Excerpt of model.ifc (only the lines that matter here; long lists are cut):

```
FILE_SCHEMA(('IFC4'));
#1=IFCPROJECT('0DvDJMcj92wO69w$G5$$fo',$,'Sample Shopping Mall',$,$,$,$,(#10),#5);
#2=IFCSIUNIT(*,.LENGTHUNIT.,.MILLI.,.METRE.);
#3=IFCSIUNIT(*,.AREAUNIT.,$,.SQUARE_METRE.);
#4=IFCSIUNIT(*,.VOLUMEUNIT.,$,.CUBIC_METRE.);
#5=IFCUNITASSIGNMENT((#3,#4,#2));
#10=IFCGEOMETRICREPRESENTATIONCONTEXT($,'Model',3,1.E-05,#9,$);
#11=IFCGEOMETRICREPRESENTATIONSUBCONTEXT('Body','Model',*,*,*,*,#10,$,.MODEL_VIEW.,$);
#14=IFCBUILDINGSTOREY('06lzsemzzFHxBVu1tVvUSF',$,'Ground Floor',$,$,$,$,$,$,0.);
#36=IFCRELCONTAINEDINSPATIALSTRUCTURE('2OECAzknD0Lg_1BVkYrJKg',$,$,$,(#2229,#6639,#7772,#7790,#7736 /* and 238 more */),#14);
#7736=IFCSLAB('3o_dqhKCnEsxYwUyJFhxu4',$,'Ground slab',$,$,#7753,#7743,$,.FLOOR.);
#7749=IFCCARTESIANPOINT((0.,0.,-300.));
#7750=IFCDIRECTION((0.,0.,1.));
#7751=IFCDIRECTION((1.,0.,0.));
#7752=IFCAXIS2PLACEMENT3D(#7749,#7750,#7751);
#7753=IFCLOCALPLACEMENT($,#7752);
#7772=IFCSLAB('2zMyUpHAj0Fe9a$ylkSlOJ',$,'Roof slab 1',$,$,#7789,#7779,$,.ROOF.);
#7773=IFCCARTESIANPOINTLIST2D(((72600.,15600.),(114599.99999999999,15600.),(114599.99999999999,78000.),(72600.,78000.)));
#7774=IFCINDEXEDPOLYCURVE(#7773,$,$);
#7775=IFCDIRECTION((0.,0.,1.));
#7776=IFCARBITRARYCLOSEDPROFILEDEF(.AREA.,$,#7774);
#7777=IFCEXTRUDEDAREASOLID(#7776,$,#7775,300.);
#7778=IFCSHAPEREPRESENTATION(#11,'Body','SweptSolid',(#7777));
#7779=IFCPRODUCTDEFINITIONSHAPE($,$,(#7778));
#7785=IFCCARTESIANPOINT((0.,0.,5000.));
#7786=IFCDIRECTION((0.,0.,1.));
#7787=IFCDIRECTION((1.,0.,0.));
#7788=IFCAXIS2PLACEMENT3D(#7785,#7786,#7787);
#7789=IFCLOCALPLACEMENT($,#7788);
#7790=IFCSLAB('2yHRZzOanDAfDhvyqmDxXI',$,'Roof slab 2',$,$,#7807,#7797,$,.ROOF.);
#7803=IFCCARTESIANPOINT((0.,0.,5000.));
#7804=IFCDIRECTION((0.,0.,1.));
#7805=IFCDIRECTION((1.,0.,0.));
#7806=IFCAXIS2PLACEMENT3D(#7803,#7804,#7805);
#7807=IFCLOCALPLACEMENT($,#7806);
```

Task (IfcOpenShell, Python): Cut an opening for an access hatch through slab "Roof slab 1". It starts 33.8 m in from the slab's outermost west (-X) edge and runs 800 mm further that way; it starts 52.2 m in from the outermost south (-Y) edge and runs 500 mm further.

```python
import numpy as np
import ifcopenshell
import ifcopenshell.api.feature
import ifcopenshell.api.geometry
import ifcopenshell.api.root
import ifcopenshell.geom
import ifcopenshell.util.placement
import ifcopenshell.util.representation
import ifcopenshell.util.shape
import ifcopenshell.util.unit

model = ifcopenshell.open("model.ifc")
unit_scale = ifcopenshell.util.unit.calculate_unit_scale(model)
settings = ifcopenshell.geom.settings()


def volume(element):
    """Net volume in cubic metres, openings subtracted."""
    shape = ifcopenshell.geom.create_shape(settings, element)
    return ifcopenshell.util.shape.get_volume(shape.geometry)


slab = model.by_guid("2zMyUpHAj0Fe9a$ylkSlOJ")
before = volume(slab)

# Extent in the slab's own axes, in metres. The edges named are its -X and -Y sides.
slab_shape = ifcopenshell.geom.create_shape(settings, slab)
vertices = ifcopenshell.util.shape.get_vertices(slab_shape.geometry)
x_min, y_min, bottom = vertices.min(axis=0)
top = vertices[:, 2].max()

opening = ifcopenshell.api.root.create_entity(model, ifc_class="IfcOpeningElement", name="Access hatch opening", predefined_type="OPENING")
context = ifcopenshell.util.representation.get_context(model, "Model", "Body", "MODEL_VIEW")
width, depth = 0.8, 0.5
outline = [(0.0, 0.0), (width, 0.0), (width, depth), (0.0, depth), (0.0, 0.0)]
# Overshoot both faces by 50 mm so the cut is clean.
shape = ifcopenshell.api.geometry.add_slab_representation(
    model, context=context, depth=top - bottom + 0.1, polyline=outline
)
ifcopenshell.api.geometry.assign_representation(model, product=opening, representation=shape)

matrix = ifcopenshell.util.placement.get_local_placement(slab.ObjectPlacement)
matrix[:, 3] = matrix @ np.append(np.array([x_min + 33.8, y_min + 52.2, bottom - 0.05]) / unit_scale, 1.0)
ifcopenshell.api.geometry.edit_object_placement(model, product=opening, matrix=matrix, is_si=False)
ifcopenshell.api.feature.add_feature(model, feature=opening, element=slab)

after = volume(slab)

print(f"slab volume {before:.3f} -> {after:.3f} m3")

model.write("model_rev.ifc")
```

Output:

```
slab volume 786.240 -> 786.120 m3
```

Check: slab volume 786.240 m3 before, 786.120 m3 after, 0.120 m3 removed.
